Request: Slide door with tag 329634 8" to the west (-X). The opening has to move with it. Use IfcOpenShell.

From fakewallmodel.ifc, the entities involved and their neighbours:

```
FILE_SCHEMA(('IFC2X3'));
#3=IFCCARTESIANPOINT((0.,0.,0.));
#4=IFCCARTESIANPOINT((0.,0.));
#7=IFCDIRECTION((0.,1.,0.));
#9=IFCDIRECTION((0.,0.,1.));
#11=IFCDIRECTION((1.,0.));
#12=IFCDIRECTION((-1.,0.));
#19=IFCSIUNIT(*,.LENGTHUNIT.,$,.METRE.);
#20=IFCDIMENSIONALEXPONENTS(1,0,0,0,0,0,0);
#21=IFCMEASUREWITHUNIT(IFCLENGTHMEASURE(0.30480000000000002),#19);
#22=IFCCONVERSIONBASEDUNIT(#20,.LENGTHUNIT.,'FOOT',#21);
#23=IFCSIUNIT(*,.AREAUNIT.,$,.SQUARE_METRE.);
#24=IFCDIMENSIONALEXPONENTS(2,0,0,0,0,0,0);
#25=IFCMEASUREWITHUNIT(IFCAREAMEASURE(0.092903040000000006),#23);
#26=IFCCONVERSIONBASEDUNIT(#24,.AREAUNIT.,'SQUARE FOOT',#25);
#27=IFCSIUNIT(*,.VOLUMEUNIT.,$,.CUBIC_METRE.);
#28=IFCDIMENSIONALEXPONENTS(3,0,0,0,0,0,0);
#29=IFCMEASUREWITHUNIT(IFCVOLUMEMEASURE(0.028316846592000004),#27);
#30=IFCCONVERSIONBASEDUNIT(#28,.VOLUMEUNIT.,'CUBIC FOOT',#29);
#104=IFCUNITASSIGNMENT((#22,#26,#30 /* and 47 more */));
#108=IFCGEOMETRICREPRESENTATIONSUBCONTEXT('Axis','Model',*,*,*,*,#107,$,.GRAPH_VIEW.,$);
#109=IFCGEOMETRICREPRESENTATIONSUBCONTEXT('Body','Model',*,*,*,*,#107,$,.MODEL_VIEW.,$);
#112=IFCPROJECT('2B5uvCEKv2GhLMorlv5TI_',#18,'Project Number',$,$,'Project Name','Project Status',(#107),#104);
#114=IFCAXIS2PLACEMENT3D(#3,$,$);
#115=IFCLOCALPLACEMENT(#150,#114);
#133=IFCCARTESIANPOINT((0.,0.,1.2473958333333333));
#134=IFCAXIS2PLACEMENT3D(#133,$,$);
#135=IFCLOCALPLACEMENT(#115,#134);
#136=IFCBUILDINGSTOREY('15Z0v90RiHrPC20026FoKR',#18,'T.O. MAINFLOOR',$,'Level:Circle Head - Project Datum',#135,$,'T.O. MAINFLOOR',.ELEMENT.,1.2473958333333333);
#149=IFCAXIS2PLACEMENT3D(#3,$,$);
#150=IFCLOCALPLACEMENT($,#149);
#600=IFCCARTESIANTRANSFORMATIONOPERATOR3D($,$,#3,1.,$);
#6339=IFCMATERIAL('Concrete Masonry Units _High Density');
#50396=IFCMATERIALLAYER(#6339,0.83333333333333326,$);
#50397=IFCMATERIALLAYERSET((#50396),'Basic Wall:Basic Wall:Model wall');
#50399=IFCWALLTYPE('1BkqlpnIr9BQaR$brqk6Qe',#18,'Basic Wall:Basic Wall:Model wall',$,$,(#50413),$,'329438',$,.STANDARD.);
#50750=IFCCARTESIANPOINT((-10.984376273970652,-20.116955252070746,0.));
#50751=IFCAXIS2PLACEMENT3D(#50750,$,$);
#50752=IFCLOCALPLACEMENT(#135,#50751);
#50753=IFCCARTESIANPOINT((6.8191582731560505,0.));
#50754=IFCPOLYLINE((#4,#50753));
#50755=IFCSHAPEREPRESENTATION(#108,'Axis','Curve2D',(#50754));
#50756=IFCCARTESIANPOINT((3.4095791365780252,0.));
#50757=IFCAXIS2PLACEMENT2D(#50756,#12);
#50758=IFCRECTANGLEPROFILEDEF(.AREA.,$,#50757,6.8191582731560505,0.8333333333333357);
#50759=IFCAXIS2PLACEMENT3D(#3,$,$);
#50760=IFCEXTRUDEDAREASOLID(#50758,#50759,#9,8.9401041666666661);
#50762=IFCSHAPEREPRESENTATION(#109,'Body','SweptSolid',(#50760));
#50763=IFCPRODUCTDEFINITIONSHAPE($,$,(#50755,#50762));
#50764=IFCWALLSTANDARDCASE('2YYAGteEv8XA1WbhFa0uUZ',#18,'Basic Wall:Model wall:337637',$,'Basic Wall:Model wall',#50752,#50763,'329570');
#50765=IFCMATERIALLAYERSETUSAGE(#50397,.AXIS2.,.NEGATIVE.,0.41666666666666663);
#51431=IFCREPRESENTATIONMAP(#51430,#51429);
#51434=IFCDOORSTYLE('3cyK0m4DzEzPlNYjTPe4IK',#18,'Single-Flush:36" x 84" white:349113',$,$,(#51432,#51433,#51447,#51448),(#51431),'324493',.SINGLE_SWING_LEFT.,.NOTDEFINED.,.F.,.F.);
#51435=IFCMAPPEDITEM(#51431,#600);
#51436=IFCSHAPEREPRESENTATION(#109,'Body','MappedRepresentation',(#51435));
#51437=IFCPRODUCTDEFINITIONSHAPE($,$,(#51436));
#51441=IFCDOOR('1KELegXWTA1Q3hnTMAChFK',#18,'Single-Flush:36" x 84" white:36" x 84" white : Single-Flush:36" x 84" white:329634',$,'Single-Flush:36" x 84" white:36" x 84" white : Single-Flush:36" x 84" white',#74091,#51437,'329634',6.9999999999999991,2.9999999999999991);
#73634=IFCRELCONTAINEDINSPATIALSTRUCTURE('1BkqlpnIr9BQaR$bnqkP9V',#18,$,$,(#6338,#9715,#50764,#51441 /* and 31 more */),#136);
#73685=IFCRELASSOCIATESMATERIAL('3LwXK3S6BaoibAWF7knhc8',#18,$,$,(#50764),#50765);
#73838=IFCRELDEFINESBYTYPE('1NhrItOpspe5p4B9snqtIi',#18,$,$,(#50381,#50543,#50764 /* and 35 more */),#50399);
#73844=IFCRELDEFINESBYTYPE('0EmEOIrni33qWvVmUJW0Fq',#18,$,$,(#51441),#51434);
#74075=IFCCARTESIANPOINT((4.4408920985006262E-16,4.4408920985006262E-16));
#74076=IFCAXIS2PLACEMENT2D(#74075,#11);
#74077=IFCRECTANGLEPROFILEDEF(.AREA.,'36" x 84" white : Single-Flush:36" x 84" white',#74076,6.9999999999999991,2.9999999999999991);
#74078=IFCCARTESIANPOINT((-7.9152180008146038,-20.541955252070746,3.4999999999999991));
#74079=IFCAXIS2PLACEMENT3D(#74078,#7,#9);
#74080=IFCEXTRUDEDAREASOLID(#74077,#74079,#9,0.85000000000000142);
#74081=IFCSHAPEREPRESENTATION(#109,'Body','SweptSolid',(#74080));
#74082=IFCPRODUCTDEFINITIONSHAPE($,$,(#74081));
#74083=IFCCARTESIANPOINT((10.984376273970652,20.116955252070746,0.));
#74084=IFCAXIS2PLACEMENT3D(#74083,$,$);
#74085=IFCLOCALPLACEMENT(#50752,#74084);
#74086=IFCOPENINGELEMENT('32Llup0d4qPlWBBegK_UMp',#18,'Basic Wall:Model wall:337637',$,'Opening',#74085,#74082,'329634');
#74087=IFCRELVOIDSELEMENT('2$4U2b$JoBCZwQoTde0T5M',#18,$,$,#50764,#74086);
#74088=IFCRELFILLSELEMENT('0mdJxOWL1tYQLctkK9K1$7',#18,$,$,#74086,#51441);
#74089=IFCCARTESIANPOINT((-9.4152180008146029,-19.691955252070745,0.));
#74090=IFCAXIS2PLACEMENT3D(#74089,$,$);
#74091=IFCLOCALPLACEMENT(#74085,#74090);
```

```python
import ifcopenshell
import ifcopenshell.api.geometry
import ifcopenshell.util.placement
import ifcopenshell.util.unit

model = ifcopenshell.open("fakewallmodel.ifc")
unit_scale = ifcopenshell.util.unit.calculate_unit_scale(model)

door = model.by_id(51441)
opening = door.FillsVoids[0].RelatingOpeningElement
wall = opening.VoidsElements[0].RelatingBuildingElement

wall_matrix = ifcopenshell.util.placement.get_local_placement(wall.ObjectPlacement)
shift = wall_matrix[:3, 0] * -8 * 0.0254 / unit_scale
before = ifcopenshell.util.placement.get_local_placement(door.ObjectPlacement)[:3, 3].copy()

# The door is placed relative to its opening, so it follows when the opening moves.
matrix = ifcopenshell.util.placement.get_local_placement(opening.ObjectPlacement)
matrix[:3, 3] += shift
ifcopenshell.api.geometry.edit_object_placement(
    model, product=opening, matrix=matrix, is_si=False, should_transform_children=True
)

after = ifcopenshell.util.placement.get_local_placement(door.ObjectPlacement)[:3, 3]
print("door moved by", (after - before).round(3) + 0.0)

model.write("fakewallmodel_v2.ifc")
```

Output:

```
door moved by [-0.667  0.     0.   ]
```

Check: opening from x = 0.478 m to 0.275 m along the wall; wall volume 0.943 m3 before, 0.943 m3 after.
